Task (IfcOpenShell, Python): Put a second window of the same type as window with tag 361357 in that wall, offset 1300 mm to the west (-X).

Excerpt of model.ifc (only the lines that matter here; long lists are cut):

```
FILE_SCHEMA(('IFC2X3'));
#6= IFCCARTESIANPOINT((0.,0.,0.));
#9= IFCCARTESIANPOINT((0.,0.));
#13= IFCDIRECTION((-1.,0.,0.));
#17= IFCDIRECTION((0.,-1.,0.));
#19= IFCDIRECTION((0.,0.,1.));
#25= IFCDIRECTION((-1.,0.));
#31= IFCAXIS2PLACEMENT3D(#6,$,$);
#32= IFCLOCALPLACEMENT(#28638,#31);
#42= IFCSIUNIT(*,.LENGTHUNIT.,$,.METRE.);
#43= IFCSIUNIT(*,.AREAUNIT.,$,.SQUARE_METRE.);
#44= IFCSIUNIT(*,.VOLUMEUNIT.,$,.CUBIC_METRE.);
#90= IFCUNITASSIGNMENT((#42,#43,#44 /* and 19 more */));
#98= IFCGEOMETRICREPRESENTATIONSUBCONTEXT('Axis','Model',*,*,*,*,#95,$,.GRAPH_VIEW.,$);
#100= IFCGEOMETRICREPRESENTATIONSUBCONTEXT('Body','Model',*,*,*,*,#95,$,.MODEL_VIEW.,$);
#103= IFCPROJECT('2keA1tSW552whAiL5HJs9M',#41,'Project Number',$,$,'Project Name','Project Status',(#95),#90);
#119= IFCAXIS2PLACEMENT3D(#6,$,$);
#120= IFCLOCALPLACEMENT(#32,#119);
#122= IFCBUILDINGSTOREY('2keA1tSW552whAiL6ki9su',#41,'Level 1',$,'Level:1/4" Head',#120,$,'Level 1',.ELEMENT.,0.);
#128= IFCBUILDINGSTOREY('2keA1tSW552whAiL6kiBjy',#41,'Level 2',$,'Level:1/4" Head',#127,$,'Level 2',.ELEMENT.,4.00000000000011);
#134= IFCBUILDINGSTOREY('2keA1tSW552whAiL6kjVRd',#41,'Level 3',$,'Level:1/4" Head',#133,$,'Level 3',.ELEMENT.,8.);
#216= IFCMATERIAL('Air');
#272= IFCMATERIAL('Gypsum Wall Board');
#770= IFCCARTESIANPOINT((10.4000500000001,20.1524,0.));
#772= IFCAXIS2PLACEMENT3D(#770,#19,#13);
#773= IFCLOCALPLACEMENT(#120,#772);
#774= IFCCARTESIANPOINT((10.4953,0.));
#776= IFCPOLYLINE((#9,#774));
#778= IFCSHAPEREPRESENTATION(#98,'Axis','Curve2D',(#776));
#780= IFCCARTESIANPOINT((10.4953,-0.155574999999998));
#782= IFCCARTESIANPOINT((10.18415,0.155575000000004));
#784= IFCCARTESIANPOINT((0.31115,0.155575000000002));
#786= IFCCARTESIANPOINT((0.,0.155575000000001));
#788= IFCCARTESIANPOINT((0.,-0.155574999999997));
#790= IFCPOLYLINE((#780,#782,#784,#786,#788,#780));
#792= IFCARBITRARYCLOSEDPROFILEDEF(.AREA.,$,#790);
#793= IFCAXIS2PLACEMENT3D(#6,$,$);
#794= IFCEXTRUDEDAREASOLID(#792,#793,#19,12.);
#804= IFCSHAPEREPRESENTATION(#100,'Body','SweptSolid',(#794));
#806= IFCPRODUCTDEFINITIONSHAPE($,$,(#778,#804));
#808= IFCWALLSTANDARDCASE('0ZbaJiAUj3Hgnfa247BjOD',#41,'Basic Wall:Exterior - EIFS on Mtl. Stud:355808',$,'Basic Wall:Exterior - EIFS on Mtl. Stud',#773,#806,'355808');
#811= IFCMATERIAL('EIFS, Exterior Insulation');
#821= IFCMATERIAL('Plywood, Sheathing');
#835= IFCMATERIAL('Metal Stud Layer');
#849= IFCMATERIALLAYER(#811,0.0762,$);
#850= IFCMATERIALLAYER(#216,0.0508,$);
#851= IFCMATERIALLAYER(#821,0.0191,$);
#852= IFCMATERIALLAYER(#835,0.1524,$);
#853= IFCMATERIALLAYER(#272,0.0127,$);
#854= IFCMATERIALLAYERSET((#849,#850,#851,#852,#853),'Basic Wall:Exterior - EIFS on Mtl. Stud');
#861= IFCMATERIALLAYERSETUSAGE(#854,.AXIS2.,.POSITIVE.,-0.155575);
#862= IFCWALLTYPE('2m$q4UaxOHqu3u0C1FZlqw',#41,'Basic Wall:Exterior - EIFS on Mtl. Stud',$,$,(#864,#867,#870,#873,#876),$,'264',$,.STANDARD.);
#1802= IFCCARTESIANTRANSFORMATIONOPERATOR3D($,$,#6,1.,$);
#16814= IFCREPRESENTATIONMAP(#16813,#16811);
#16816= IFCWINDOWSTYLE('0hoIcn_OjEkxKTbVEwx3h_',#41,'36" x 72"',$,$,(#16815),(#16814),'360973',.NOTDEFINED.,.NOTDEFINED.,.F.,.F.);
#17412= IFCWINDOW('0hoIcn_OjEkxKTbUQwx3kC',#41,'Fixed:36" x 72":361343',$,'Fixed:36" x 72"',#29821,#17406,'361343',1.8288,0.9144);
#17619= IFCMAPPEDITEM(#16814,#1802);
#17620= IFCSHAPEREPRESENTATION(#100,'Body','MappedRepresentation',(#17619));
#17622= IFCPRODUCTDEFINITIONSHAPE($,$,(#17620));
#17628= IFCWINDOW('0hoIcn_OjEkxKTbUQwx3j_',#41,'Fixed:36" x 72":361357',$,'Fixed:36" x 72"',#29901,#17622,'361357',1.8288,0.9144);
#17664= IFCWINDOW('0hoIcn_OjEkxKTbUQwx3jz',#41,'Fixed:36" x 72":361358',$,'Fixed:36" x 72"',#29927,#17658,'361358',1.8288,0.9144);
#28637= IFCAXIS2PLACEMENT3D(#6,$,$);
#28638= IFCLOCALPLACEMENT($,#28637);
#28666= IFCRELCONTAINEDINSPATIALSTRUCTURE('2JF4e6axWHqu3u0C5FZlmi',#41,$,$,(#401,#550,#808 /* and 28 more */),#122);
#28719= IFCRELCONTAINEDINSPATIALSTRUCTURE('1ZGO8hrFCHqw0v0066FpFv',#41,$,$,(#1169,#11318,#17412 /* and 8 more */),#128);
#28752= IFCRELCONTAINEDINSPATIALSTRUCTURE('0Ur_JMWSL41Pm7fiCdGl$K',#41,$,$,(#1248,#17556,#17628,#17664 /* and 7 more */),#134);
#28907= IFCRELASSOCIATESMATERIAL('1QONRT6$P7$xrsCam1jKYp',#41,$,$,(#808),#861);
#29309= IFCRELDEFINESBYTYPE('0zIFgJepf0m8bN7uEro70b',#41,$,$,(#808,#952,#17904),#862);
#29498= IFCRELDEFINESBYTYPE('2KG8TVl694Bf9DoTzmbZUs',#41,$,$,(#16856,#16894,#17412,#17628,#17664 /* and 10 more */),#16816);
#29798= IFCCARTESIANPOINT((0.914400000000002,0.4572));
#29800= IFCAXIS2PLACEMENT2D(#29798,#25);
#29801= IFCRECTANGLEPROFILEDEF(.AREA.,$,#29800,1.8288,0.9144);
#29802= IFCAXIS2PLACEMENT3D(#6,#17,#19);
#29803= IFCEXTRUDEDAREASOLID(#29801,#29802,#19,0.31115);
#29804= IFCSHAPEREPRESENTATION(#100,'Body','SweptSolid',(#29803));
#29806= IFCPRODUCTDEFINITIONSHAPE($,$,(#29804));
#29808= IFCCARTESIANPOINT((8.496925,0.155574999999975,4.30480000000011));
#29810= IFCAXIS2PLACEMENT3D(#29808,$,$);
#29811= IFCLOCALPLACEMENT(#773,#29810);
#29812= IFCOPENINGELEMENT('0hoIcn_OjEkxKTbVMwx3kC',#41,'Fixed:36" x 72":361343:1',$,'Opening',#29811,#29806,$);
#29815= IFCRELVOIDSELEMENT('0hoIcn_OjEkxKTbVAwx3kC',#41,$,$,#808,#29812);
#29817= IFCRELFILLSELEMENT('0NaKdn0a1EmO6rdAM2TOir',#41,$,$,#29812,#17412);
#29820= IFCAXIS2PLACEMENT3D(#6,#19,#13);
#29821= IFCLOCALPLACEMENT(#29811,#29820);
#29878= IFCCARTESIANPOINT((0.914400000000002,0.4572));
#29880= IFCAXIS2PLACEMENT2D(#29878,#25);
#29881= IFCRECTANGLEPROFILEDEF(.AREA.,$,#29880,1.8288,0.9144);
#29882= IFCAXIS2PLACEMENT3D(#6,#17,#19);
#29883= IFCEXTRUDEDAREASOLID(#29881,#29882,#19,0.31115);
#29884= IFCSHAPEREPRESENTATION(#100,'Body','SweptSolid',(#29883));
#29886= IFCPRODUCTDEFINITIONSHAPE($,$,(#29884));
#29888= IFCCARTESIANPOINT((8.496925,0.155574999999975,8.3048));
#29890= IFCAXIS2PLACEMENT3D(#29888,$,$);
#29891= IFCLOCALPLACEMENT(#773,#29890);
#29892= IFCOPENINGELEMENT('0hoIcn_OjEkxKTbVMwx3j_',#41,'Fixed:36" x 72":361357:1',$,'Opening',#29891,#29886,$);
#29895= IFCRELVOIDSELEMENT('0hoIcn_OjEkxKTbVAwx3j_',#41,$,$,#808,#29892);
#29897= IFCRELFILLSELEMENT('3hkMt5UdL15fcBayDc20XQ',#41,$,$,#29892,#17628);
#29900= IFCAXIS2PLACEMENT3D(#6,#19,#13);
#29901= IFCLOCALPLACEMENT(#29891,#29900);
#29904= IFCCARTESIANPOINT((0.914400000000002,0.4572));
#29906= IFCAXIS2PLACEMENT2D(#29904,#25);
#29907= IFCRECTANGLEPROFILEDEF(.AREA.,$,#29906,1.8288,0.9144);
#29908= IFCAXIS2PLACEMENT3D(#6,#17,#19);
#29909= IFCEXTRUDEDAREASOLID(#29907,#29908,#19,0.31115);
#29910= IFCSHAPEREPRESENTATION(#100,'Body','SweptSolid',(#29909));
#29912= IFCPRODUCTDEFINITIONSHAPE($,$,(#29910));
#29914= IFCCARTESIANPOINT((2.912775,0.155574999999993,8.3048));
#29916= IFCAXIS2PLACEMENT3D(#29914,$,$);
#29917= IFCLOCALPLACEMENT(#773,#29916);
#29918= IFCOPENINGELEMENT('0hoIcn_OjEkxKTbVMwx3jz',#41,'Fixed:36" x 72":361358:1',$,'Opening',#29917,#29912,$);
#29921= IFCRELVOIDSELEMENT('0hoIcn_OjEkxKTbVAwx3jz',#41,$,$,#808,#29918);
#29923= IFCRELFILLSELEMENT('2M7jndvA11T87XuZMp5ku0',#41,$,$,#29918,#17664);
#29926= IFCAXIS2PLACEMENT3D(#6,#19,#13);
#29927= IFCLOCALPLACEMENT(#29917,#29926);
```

```python
import ifcopenshell
import ifcopenshell.api.feature
import ifcopenshell.api.geometry
import ifcopenshell.api.root
import ifcopenshell.geom
import ifcopenshell.util.element
import ifcopenshell.util.placement
import ifcopenshell.util.shape

model = ifcopenshell.open("model.ifc")
settings = ifcopenshell.geom.settings()


def volume(element):
    """Net volume in cubic metres, openings subtracted."""
    shape = ifcopenshell.geom.create_shape(settings, element)
    return ifcopenshell.util.shape.get_volume(shape.geometry)


def reuse_history(source, copy):
    """copy_class also copies each property set's owner history, people and application; keep the originals."""
    for rel in copy.IsDefinedBy:
        if rel.is_a("IfcRelDefinesByProperties") and (history := rel.RelatingPropertyDefinition.OwnerHistory):
            rel.RelatingPropertyDefinition.OwnerHistory = source.OwnerHistory
            ifcopenshell.util.element.remove_deep2(model, history)


window = model.by_guid("0hoIcn_OjEkxKTbUQwx3j_")
opening = window.FillsVoids[0].RelatingOpeningElement
wall = opening.VoidsElements[0].RelatingBuildingElement
before = volume(wall)
shift = ifcopenshell.util.placement.get_local_placement(wall.ObjectPlacement)[:3, 0] * 1.3

# copy_class copies the void relationship, type, container and properties, but no geometry.
new_opening = ifcopenshell.api.root.copy_class(model, product=opening)
new_opening.Representation = ifcopenshell.util.element.copy_deep(
    model, opening.Representation, exclude=["IfcGeometricRepresentationContext", "IfcRepresentationMap"]
)
new_opening.Name = 'Fixed:36" x 72"'
new_window = ifcopenshell.api.root.copy_class(model, product=window)
new_window.Representation = ifcopenshell.util.element.copy_deep(
    model, window.Representation, exclude=["IfcGeometricRepresentationContext", "IfcRepresentationMap"]
)
new_window.Name = 'Fixed:36" x 72"'
new_window.Tag = None
reuse_history(window, new_window)
fills = ifcopenshell.api.feature.add_filling(model, opening=new_opening, element=new_window)
fills.OwnerHistory = new_window.OwnerHistory  # required in IFC2X3

for old, new in ((opening, new_opening), (window, new_window)):
    matrix = ifcopenshell.util.placement.get_local_placement(old.ObjectPlacement)
    matrix[:3, 3] += shift
    ifcopenshell.api.geometry.edit_object_placement(model, product=new, matrix=matrix, is_si=False)

after = volume(wall)

print(f"wall volume {before:.3f} -> {after:.3f} m3")

model.write("model_updated.ifc")
```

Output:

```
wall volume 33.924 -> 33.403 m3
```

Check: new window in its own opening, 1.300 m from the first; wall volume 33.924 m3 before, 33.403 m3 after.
